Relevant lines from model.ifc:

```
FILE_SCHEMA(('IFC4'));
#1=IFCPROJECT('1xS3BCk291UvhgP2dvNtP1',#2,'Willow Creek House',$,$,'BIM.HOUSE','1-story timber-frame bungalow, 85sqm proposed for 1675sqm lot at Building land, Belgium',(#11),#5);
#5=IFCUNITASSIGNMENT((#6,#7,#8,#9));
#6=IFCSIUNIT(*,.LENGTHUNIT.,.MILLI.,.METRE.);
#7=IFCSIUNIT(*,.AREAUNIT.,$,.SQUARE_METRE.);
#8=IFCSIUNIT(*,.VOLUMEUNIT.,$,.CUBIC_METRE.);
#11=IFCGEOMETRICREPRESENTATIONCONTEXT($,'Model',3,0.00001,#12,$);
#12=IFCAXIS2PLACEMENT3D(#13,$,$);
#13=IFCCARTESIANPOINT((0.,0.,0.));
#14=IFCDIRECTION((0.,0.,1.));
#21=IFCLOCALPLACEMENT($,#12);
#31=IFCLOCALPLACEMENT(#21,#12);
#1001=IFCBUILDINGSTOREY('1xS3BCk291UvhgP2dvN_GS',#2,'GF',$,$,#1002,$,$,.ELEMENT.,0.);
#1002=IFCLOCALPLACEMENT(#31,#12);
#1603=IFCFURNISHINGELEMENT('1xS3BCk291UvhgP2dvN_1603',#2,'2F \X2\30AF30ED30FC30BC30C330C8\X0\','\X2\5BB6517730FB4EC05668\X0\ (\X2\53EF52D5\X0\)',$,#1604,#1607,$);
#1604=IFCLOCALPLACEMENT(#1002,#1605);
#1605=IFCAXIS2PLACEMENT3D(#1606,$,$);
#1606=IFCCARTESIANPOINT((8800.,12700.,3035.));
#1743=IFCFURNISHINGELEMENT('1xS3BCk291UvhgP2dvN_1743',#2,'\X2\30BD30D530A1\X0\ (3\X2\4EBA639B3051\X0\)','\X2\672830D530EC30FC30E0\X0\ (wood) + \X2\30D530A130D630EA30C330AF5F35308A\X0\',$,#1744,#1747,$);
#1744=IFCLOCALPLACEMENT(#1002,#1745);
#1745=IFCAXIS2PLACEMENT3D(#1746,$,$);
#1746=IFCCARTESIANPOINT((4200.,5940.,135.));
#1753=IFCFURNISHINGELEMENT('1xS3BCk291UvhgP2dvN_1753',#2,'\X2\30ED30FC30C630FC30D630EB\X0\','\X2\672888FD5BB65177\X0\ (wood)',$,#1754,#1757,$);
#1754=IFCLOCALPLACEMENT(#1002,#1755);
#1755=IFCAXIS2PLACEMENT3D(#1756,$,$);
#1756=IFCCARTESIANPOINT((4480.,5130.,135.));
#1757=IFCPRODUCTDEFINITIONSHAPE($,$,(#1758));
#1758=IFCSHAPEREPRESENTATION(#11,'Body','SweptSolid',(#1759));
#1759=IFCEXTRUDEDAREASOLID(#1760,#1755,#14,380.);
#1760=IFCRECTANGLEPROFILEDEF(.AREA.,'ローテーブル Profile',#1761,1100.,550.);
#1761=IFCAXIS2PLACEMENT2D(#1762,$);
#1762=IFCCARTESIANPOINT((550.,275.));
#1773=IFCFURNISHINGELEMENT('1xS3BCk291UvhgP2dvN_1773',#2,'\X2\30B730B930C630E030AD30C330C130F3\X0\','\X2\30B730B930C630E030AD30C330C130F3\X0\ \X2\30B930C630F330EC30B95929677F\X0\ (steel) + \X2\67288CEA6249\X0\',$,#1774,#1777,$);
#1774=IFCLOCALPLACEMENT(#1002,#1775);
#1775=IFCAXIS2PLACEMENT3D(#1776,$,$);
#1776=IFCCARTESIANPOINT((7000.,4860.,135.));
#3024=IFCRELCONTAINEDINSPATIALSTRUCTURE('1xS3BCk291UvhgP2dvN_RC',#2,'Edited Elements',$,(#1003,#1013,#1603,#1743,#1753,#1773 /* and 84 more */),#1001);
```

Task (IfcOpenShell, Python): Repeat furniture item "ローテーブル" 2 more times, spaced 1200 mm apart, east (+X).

```python
import numpy as np
import ifcopenshell
import ifcopenshell.api.geometry
import ifcopenshell.api.root
import ifcopenshell.util.element
import ifcopenshell.util.placement
import ifcopenshell.util.unit

model = ifcopenshell.open("model.ifc")
unit_scale = ifcopenshell.util.unit.calculate_unit_scale(model)


def reuse_history(source, copy):
    """copy_class also copies each property set's owner history, people and application; keep the originals."""
    for rel in copy.IsDefinedBy:
        if rel.is_a("IfcRelDefinesByProperties") and (history := rel.RelatingPropertyDefinition.OwnerHistory):
            rel.RelatingPropertyDefinition.OwnerHistory = source.OwnerHistory
            ifcopenshell.util.element.remove_deep2(model, history)


source = model.by_guid("1xS3BCk291UvhgP2dvN_1753")
base = ifcopenshell.util.placement.get_local_placement(source.ObjectPlacement)
step = np.array([1.0, 0.0, 0.0]) * 1.2 / unit_scale

for i in range(1, 3):
    copy = ifcopenshell.api.root.copy_class(model, product=source)
    copy.Representation = ifcopenshell.util.element.copy_deep(
        model, source.Representation, exclude=["IfcGeometricRepresentationContext", "IfcRepresentationMap"]
    )
    reuse_history(source, copy)
    matrix = base.copy()
    matrix[:3, 3] += i * step
    print("added at", matrix[:3, 3].round(3) + 0.0)
    ifcopenshell.api.geometry.edit_object_placement(model, product=copy, matrix=matrix, is_si=False)

model.write("model_rev.ifc")
```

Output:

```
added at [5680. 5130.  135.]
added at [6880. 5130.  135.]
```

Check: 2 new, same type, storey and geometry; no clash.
